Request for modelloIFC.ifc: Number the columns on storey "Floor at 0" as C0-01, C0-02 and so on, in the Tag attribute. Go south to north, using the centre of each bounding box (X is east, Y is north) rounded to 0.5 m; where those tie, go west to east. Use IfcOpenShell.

First a look at what the model holds.

```python
import ifcopenshell
import ifcopenshell.util.element
import ifcopenshell.util.placement

model = ifcopenshell.open("modelloIFC.ifc")
print(model.schema)
storey = next(s for s in model.by_type("IfcBuildingStorey") if s.Name == "Floor at 0")
columns = [e for e in ifcopenshell.util.element.get_decomposition(storey) if e.is_a("IfcColumn")]
for e in sorted(columns, key=lambda e: e.id()):
    origin = ifcopenshell.util.placement.get_local_placement(e.ObjectPlacement)[:3, 3]
    print(e.id(), e.Tag, e.Name, origin.round(2) + 0.0, sep=" | ")
```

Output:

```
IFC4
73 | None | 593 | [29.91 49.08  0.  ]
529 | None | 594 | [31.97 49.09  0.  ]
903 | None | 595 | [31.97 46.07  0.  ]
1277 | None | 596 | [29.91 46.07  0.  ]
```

```python
import ifcopenshell
import ifcopenshell.geom
import ifcopenshell.util.element
import ifcopenshell.util.shape

model = ifcopenshell.open("modelloIFC.ifc")
settings = ifcopenshell.geom.settings()
settings.set("use-world-coords", True)


def centre(element):
    shape = ifcopenshell.geom.create_shape(settings, element)
    return ifcopenshell.util.shape.get_bbox_centroid(shape.geometry)


storey = next(s for s in model.by_type("IfcBuildingStorey") if s.Name == "Floor at 0")
columns = [e for e in ifcopenshell.util.element.get_decomposition(storey) if e.is_a("IfcColumn")]

# Insertion points can sit at a corner or the storey origin, so sort by the geometry (in metres).
centres = {e: centre(e) for e in columns}
columns.sort(key=lambda e: (round(centres[e][1] / 0.5), centres[e][0]))

for i, e in enumerate(columns, start=1):
    number = f"C0-{i:02d}"
    e.Tag = number
    print(e.id(), number)

model.write("modelloIFC_edited.ifc")
```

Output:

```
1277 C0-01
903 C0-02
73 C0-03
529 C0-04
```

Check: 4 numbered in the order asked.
